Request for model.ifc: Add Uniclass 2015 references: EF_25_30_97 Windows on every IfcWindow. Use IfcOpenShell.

First a look at what the model holds.

```python
import ifcopenshell

model = ifcopenshell.open("model.ifc")
print(model.schema)
print("classifications:", [c.Name for c in model.by_type("IfcClassification")])
for ifc_class in ("IfcDoor", "IfcRoof", "IfcStair", "IfcWall", "IfcWindow"):
    print(ifc_class, len(model.by_type(ifc_class)))
```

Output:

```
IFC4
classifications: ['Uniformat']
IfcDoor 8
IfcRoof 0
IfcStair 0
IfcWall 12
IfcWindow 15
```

```python
import ifcopenshell
import ifcopenshell.api.classification

model = ifcopenshell.open("model.ifc")

system = ifcopenshell.api.classification.add_classification(model, classification="Uniclass 2015")

codes = {
    "IfcWindow": ("EF_25_30_97", "Windows"),
}
for ifc_class, (code, name) in codes.items():
    products = model.by_type(ifc_class)
    ifcopenshell.api.classification.add_reference(
        model, products=products, classification=system, identification=code, name=name
    )
    print(code, len(products))

model.write("model-out.ifc")
```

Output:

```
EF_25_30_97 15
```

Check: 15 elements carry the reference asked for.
